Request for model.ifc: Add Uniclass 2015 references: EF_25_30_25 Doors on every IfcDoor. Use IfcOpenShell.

First a look at what the model holds.

```python
import ifcopenshell

model = ifcopenshell.open("model.ifc")
print(model.schema)
print("classifications:", [c.Name for c in model.by_type("IfcClassification")])
for ifc_class in ("IfcDoor", "IfcRoof", "IfcStair", "IfcWall", "IfcWindow"):
    print(ifc_class, len(model.by_type(ifc_class)))
```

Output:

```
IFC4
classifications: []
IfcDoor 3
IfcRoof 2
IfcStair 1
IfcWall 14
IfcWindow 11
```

```python
import ifcopenshell
import ifcopenshell.api.classification

model = ifcopenshell.open("model.ifc")

system = ifcopenshell.api.classification.add_classification(model, classification="Uniclass 2015")

codes = {
    "IfcDoor": ("EF_25_30_25", "Doors"),
}
for ifc_class, (code, name) in codes.items():
    products = model.by_type(ifc_class)
    ifcopenshell.api.classification.add_reference(
        model, products=products, classification=system, identification=code, name=name
    )
    print(code, len(products))

model.write("model_edited.ifc")
```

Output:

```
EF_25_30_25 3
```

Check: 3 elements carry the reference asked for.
